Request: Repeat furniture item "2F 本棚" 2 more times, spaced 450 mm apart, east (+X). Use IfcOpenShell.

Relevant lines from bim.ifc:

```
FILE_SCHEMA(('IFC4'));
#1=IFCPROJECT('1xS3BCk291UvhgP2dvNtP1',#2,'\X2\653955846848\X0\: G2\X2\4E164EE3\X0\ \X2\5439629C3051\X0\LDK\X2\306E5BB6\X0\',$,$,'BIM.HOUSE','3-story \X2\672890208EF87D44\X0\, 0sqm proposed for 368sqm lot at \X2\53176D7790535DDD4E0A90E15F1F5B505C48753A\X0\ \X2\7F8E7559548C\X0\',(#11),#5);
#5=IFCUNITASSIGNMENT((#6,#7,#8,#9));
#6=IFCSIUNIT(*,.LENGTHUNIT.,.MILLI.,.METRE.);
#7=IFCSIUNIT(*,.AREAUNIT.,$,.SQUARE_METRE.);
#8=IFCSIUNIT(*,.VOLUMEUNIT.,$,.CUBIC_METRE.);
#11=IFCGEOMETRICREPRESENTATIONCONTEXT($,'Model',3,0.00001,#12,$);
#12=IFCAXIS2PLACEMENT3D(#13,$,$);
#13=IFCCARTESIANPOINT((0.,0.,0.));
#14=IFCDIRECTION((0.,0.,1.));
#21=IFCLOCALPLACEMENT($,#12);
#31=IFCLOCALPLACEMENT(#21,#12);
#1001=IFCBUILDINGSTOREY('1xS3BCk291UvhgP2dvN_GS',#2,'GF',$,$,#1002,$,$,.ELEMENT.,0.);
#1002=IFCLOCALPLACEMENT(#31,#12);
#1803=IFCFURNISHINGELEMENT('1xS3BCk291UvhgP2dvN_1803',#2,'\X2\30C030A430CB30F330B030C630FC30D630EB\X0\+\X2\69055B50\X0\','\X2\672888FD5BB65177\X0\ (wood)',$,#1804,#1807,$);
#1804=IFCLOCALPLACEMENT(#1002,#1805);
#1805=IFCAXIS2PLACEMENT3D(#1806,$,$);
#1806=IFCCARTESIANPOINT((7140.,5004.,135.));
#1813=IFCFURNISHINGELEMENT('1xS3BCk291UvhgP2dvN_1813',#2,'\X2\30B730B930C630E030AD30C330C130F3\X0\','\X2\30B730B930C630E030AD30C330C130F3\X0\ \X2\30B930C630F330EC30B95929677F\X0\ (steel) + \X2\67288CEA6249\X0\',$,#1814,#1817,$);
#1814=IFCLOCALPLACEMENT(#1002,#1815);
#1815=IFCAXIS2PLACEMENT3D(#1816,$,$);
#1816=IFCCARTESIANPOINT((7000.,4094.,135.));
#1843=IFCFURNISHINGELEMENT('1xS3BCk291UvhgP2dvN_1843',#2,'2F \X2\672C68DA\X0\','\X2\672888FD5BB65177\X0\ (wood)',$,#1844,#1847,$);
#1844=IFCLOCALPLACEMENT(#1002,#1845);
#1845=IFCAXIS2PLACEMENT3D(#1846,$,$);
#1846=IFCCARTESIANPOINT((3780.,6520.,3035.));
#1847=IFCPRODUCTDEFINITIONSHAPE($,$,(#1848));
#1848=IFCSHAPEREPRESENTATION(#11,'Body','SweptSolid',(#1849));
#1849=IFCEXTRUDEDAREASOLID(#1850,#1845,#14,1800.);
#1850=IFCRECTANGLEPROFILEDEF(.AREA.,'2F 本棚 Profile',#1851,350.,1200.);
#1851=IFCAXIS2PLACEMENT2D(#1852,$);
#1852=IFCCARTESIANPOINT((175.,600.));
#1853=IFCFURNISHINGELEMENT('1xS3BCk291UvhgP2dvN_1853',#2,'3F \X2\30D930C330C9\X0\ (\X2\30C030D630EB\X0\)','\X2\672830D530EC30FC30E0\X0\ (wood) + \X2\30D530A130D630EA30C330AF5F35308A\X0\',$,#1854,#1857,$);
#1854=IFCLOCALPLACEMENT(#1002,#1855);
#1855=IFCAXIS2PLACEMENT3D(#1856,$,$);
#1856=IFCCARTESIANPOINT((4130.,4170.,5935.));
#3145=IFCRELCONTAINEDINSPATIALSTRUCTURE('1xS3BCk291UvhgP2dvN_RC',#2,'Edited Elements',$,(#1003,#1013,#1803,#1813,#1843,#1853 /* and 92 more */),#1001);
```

```python
import numpy as np
import ifcopenshell
import ifcopenshell.api.geometry
import ifcopenshell.api.root
import ifcopenshell.util.element
import ifcopenshell.util.placement
import ifcopenshell.util.unit

model = ifcopenshell.open("bim.ifc")
unit_scale = ifcopenshell.util.unit.calculate_unit_scale(model)


def reuse_history(source, copy):
    """copy_class also copies each property set's owner history, people and application; keep the originals."""
    for rel in copy.IsDefinedBy:
        if rel.is_a("IfcRelDefinesByProperties") and (history := rel.RelatingPropertyDefinition.OwnerHistory):
            rel.RelatingPropertyDefinition.OwnerHistory = source.OwnerHistory
            ifcopenshell.util.element.remove_deep2(model, history)


source = model.by_id(1843)
base = ifcopenshell.util.placement.get_local_placement(source.ObjectPlacement)
step = np.array([1.0, 0.0, 0.0]) * 0.45 / unit_scale

for i in range(1, 3):
    copy = ifcopenshell.api.root.copy_class(model, product=source)
    copy.Representation = ifcopenshell.util.element.copy_deep(
        model, source.Representation, exclude=["IfcGeometricRepresentationContext", "IfcRepresentationMap"]
    )
    reuse_history(source, copy)
    matrix = base.copy()
    matrix[:3, 3] += i * step
    print("added at", matrix[:3, 3].round(3) + 0.0)
    ifcopenshell.api.geometry.edit_object_placement(model, product=copy, matrix=matrix, is_si=False)

model.write("bim_rev.ifc")
```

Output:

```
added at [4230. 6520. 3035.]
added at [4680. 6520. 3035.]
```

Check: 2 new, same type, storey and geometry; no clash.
